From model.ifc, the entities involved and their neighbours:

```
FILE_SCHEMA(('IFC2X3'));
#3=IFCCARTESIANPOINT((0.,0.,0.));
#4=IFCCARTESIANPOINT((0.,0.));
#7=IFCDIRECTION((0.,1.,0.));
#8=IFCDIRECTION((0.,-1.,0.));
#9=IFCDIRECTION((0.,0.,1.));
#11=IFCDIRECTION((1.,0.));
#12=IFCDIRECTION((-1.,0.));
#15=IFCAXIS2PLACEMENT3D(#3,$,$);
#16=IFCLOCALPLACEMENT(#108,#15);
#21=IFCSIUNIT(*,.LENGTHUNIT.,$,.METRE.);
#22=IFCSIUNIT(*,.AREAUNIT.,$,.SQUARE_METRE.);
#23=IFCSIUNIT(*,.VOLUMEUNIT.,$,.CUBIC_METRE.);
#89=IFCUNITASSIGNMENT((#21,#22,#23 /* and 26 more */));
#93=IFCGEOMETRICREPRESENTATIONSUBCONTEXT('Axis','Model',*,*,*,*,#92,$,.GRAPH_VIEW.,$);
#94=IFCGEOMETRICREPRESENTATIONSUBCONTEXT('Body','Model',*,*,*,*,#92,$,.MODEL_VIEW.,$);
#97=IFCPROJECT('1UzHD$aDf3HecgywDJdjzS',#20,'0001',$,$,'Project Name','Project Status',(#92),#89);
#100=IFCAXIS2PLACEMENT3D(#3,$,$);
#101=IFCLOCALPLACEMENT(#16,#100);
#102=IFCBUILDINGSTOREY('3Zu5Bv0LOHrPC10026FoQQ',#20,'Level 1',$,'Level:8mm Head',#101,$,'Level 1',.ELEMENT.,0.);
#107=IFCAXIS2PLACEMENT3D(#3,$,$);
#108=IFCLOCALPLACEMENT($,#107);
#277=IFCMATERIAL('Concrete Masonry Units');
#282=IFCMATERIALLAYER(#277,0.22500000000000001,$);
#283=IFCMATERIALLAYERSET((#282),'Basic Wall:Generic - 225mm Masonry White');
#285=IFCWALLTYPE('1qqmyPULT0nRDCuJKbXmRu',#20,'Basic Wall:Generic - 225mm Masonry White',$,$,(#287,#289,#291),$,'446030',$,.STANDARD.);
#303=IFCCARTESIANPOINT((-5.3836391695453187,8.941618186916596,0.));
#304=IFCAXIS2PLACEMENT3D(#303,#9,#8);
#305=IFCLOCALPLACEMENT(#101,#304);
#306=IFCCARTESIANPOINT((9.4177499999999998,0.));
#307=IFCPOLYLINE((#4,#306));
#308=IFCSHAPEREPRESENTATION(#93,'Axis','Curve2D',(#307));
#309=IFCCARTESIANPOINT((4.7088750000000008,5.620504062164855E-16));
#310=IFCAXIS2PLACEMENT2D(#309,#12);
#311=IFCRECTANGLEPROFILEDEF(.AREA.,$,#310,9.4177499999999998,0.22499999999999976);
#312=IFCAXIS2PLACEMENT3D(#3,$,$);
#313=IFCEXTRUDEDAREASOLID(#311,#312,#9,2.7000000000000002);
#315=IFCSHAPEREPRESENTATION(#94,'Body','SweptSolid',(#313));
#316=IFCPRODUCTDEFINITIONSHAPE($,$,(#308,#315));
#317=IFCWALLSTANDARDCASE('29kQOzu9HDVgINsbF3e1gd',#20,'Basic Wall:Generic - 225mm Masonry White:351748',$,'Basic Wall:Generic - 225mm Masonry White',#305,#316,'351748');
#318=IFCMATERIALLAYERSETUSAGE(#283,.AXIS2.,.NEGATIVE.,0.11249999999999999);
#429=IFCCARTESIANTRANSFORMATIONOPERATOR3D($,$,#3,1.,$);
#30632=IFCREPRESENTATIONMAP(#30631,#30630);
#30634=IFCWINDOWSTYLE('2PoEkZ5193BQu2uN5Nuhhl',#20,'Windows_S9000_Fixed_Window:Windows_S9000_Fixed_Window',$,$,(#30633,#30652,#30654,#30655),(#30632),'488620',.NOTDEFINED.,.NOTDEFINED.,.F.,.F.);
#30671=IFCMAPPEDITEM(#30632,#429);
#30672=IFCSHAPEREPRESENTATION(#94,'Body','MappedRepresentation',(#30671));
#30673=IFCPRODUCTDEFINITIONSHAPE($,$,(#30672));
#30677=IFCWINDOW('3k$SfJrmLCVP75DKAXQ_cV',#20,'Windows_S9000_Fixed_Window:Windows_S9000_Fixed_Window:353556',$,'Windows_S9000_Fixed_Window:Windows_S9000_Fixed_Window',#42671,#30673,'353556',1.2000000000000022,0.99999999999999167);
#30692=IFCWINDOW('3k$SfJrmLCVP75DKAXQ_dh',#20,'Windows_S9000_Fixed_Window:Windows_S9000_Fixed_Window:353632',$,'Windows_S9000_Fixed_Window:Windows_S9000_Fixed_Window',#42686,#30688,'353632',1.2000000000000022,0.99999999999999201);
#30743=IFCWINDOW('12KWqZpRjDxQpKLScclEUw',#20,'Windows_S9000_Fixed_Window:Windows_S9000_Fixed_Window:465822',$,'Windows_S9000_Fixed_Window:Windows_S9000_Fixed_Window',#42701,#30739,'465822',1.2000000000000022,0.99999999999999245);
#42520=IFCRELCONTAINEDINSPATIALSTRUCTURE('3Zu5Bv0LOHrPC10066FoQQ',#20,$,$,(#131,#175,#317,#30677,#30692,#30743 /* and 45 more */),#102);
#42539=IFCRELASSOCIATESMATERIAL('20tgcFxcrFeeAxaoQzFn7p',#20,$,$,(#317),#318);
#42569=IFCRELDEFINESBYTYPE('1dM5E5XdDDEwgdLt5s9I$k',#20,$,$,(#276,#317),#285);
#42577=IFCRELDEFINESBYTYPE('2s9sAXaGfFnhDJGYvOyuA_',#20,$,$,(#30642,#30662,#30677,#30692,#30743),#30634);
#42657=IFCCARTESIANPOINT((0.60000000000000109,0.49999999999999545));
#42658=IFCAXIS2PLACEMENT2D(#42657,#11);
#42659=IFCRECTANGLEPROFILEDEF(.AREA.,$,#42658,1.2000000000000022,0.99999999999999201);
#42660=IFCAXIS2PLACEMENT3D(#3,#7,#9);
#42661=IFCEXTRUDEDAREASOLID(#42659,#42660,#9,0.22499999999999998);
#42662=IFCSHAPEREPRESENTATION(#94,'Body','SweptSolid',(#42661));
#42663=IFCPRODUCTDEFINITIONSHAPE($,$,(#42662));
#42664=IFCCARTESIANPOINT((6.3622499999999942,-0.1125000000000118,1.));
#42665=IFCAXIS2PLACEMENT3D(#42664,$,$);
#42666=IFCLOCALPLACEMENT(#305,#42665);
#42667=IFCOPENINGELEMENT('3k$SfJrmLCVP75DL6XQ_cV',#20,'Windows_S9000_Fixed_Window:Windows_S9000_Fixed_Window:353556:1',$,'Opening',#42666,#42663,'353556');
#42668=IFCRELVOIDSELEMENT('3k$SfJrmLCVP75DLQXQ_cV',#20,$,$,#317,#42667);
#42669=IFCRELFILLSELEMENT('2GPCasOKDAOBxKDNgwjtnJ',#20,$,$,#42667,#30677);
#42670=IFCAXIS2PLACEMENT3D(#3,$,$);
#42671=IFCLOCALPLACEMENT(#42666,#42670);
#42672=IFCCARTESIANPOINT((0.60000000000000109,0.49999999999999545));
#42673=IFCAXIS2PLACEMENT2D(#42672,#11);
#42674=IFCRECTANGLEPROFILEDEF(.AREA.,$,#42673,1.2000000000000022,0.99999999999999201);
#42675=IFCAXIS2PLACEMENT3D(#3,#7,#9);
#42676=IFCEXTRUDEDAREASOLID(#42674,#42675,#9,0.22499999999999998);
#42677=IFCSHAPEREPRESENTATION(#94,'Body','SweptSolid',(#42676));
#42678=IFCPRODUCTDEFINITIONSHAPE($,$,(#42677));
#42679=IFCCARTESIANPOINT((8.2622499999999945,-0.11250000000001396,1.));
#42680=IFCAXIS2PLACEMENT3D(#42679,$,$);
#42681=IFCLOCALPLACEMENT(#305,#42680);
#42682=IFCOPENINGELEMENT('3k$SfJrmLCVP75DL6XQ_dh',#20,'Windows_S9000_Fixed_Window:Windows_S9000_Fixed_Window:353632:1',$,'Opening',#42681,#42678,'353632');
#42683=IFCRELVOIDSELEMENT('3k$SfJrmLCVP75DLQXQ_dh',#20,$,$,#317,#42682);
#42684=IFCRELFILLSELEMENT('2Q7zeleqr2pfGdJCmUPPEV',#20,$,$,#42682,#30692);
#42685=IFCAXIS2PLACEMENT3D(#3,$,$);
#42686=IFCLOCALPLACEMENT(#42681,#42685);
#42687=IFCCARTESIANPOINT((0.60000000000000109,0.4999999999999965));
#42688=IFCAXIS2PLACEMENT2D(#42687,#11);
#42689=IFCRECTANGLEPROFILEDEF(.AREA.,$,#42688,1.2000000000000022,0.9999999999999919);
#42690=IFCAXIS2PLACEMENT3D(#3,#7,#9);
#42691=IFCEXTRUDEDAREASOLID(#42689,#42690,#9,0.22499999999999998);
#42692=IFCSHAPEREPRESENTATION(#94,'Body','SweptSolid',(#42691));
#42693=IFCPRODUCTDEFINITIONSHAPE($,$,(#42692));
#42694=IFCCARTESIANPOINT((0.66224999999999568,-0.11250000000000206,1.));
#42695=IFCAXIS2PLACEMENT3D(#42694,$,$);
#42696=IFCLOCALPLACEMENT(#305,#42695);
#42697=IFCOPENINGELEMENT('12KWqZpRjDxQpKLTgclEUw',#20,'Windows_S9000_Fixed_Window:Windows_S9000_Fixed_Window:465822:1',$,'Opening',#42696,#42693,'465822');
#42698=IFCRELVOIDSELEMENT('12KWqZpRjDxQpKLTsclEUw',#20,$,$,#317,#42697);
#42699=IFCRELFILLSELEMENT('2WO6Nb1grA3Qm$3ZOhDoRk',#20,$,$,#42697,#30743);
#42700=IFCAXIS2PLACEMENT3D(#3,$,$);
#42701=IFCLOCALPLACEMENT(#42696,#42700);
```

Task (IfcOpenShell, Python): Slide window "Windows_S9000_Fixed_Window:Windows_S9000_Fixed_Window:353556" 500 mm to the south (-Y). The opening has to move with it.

```python
import ifcopenshell
import ifcopenshell.api.geometry
import ifcopenshell.util.placement

model = ifcopenshell.open("model.ifc")

window = model.by_id(30677)
opening = window.FillsVoids[0].RelatingOpeningElement
wall = opening.VoidsElements[0].RelatingBuildingElement

wall_matrix = ifcopenshell.util.placement.get_local_placement(wall.ObjectPlacement)
shift = wall_matrix[:3, 0] * 0.5
before = ifcopenshell.util.placement.get_local_placement(window.ObjectPlacement)[:3, 3].copy()

# The window is placed relative to its opening, so it follows when the opening moves.
matrix = ifcopenshell.util.placement.get_local_placement(opening.ObjectPlacement)
matrix[:3, 3] += shift
ifcopenshell.api.geometry.edit_object_placement(
    model, product=opening, matrix=matrix, is_si=False, should_transform_children=True
)

after = ifcopenshell.util.placement.get_local_placement(window.ObjectPlacement)[:3, 3]
print("window moved by", (after - before).round(3) + 0.0)

model.write("model_updated.ifc")
```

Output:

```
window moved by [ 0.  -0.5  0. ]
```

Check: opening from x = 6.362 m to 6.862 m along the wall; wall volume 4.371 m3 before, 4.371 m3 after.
